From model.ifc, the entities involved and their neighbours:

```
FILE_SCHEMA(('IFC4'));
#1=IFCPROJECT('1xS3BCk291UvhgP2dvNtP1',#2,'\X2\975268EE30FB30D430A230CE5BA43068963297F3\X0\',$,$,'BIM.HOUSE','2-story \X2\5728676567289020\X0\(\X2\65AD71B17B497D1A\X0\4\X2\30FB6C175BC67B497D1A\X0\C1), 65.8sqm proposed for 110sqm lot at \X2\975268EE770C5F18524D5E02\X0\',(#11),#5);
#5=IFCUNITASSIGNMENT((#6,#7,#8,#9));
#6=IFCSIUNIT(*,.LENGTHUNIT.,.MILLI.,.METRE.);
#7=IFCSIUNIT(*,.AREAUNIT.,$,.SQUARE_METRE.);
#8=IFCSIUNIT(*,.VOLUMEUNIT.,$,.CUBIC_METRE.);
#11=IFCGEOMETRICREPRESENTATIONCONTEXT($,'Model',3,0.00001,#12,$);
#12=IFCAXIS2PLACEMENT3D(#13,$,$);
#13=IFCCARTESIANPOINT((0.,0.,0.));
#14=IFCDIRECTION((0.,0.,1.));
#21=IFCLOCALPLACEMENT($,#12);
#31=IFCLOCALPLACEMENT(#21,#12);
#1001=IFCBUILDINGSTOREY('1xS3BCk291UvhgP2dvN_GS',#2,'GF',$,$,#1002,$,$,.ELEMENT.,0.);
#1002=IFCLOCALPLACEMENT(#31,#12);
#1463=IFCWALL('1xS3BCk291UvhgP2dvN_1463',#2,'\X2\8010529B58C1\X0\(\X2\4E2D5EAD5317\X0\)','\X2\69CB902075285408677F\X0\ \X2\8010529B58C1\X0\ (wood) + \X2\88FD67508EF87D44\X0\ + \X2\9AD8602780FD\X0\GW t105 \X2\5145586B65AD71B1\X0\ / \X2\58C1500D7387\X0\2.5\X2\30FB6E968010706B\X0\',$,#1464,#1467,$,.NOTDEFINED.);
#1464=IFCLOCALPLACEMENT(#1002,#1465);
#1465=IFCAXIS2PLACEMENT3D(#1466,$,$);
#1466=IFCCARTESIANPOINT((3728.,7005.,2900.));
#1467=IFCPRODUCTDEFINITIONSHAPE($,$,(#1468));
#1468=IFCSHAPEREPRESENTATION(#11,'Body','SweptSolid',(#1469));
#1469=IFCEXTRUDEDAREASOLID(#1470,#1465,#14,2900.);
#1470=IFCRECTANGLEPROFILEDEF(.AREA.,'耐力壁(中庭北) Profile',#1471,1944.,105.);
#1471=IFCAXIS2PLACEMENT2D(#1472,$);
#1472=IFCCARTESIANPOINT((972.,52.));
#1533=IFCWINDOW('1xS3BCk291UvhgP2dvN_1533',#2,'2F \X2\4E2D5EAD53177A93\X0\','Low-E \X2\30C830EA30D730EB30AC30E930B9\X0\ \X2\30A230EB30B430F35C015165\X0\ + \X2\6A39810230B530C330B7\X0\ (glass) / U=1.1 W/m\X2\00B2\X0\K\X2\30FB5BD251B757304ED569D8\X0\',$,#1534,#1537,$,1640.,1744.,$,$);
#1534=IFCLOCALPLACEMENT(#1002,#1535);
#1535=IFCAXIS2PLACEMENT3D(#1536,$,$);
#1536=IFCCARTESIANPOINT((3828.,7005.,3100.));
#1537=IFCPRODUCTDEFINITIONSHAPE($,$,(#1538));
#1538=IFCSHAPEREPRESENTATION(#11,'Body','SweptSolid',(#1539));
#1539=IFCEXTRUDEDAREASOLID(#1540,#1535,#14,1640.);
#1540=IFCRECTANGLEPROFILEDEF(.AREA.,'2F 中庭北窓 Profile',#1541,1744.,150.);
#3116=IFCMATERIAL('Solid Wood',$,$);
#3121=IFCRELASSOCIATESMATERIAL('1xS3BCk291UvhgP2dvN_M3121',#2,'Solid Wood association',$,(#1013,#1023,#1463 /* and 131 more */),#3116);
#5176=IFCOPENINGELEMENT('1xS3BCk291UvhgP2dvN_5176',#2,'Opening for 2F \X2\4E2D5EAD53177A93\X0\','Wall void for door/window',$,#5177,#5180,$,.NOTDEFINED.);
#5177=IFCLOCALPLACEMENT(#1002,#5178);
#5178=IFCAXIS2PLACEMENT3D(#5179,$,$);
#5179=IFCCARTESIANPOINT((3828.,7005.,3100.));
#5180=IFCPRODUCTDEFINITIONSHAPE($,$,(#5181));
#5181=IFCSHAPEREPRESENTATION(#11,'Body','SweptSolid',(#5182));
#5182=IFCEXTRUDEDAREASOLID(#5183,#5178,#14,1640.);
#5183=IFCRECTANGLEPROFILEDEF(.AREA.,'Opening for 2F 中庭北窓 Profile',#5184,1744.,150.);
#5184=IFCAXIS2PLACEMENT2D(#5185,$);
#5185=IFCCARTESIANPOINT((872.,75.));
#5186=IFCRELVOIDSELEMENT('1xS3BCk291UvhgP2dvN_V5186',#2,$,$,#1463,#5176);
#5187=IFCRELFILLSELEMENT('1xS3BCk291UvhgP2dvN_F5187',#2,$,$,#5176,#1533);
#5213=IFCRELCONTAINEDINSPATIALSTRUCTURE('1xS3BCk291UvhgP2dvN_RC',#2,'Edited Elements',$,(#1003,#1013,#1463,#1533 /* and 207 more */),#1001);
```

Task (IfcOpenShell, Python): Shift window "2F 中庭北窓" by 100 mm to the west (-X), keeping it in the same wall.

```python
import ifcopenshell
import ifcopenshell.api.geometry
import ifcopenshell.util.placement
import ifcopenshell.util.unit

model = ifcopenshell.open("model.ifc")
unit_scale = ifcopenshell.util.unit.calculate_unit_scale(model)

window = model.by_guid("1xS3BCk291UvhgP2dvN_1533")
opening = window.FillsVoids[0].RelatingOpeningElement
wall = opening.VoidsElements[0].RelatingBuildingElement

wall_matrix = ifcopenshell.util.placement.get_local_placement(wall.ObjectPlacement)
shift = wall_matrix[:3, 0] * -0.1 / unit_scale
before = ifcopenshell.util.placement.get_local_placement(window.ObjectPlacement)[:3, 3].copy()

# The window is not placed relative to its opening, so move both.
for product in (opening, window):
    matrix = ifcopenshell.util.placement.get_local_placement(product.ObjectPlacement)
    matrix[:3, 3] += shift
    ifcopenshell.api.geometry.edit_object_placement(model, product=product, matrix=matrix, is_si=False)

after = ifcopenshell.util.placement.get_local_placement(window.ObjectPlacement)[:3, 3]
print("window moved by", (after - before).round(3) + 0.0)

model.write("model-out.ifc")
```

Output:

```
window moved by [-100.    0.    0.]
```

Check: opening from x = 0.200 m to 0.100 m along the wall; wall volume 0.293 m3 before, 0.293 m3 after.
